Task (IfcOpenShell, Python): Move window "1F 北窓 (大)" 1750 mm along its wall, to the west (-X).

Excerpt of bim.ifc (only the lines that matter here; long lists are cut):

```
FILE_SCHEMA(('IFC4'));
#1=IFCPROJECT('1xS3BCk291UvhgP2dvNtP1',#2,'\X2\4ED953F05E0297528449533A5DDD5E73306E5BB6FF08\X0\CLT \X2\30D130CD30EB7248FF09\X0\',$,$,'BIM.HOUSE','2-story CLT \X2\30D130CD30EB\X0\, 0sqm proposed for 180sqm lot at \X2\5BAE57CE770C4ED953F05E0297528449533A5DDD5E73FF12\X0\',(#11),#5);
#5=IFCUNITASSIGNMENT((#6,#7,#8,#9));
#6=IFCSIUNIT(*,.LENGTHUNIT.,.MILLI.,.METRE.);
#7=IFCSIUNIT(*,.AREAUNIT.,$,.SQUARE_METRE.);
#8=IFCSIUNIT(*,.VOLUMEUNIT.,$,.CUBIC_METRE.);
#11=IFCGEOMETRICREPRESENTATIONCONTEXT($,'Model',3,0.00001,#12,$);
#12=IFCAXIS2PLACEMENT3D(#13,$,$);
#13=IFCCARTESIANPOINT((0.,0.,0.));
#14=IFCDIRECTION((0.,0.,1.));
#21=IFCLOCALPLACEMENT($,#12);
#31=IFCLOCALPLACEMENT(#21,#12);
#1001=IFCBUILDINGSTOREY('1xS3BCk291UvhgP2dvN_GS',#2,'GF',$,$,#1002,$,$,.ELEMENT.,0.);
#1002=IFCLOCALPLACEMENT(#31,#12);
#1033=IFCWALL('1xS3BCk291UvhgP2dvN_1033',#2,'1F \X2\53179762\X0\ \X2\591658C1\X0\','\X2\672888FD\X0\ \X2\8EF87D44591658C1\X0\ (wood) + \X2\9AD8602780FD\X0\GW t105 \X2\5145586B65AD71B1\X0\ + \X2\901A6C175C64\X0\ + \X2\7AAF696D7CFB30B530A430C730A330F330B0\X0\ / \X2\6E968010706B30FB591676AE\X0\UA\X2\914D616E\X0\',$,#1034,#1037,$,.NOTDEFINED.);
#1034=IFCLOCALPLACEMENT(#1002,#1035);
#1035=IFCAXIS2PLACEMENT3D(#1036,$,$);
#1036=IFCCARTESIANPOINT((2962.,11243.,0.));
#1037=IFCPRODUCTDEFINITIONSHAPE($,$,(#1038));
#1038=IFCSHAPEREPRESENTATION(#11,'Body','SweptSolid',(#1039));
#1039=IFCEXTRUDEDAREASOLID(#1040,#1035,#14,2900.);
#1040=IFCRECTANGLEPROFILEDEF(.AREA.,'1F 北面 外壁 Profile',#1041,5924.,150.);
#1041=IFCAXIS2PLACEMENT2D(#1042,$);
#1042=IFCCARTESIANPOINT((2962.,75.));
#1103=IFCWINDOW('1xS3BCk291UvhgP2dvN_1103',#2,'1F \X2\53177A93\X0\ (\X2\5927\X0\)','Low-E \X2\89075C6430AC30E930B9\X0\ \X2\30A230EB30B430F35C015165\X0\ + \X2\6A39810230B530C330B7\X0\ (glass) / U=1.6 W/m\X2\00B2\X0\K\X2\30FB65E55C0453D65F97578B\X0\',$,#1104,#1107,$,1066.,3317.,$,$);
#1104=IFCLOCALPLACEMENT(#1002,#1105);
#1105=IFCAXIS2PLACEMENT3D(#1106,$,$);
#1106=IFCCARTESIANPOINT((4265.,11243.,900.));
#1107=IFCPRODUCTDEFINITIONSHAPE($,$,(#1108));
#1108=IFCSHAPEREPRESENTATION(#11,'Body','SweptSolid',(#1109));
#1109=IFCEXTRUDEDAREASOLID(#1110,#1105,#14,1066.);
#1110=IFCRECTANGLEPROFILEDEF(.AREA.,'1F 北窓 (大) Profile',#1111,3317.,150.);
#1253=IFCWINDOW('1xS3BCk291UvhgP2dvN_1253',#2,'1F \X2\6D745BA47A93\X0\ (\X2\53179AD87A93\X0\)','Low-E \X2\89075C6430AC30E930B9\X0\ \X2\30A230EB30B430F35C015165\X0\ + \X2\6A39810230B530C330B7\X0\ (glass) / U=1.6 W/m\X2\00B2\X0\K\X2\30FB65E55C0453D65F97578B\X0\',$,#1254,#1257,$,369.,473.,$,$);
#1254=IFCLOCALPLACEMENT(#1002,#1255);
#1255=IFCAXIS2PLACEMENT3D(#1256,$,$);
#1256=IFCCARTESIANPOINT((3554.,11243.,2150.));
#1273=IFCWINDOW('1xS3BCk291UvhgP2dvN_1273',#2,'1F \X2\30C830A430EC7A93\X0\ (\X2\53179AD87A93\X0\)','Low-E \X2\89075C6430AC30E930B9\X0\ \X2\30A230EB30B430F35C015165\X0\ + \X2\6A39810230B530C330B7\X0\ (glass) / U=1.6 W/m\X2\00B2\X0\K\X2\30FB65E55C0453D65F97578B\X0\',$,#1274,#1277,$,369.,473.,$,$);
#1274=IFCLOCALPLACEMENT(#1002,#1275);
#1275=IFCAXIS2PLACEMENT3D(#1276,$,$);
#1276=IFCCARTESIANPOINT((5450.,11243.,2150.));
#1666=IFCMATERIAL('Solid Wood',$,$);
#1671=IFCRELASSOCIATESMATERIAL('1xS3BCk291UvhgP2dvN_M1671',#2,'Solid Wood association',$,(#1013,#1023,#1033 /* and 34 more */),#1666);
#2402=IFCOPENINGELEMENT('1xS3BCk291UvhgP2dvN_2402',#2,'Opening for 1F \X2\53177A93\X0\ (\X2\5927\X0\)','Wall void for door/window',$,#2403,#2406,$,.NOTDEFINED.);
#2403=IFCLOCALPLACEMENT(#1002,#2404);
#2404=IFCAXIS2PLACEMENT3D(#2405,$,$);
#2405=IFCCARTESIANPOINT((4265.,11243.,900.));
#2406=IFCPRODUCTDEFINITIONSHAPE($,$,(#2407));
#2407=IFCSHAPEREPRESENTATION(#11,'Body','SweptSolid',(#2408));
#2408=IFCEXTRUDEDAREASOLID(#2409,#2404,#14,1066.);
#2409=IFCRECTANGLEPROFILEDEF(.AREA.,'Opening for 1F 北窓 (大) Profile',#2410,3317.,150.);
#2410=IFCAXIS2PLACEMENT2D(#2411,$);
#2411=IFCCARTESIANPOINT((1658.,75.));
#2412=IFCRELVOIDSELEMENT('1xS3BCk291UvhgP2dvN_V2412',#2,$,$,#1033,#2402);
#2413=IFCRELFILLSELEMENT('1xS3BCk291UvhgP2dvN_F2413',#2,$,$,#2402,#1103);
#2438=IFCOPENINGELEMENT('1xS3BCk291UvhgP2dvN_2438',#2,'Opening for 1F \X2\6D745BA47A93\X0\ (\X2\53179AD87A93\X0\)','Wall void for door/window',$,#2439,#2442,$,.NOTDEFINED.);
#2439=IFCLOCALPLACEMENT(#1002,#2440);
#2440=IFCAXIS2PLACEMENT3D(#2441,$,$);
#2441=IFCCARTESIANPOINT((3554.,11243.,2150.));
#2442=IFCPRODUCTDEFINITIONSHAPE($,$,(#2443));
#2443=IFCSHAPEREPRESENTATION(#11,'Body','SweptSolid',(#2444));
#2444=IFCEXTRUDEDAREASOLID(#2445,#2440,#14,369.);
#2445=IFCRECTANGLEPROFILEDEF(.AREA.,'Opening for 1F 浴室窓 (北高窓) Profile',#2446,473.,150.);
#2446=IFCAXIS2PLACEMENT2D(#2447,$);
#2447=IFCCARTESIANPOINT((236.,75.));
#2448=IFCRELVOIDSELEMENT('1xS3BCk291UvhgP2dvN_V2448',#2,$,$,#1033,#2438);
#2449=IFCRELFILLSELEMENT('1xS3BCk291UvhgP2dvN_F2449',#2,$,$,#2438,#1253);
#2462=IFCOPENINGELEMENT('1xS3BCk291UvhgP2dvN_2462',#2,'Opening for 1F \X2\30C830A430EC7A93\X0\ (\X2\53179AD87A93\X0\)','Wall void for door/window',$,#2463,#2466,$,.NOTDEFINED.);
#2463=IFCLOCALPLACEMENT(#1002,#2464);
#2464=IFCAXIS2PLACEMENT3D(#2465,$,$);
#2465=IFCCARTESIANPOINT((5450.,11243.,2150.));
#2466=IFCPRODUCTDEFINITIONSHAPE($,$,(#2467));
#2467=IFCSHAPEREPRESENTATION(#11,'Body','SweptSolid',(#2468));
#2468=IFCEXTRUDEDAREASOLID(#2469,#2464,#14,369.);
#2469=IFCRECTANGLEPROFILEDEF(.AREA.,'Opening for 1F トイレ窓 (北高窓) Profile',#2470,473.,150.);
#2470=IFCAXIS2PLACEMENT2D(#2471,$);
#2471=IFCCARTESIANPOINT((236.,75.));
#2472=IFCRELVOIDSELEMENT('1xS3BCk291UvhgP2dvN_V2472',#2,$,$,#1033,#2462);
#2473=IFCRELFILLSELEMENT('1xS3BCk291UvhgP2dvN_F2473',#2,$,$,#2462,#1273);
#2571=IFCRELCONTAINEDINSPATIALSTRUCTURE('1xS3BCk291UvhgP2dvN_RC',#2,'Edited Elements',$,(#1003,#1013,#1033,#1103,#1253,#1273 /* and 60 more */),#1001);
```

```python
import ifcopenshell
import ifcopenshell.api.geometry
import ifcopenshell.util.placement
import ifcopenshell.util.unit

model = ifcopenshell.open("bim.ifc")
unit_scale = ifcopenshell.util.unit.calculate_unit_scale(model)

window = model.by_guid("1xS3BCk291UvhgP2dvN_1103")
opening = window.FillsVoids[0].RelatingOpeningElement
wall = opening.VoidsElements[0].RelatingBuildingElement

wall_matrix = ifcopenshell.util.placement.get_local_placement(wall.ObjectPlacement)
shift = wall_matrix[:3, 0] * -1.75 / unit_scale
before = ifcopenshell.util.placement.get_local_placement(window.ObjectPlacement)[:3, 3].copy()

# The window is not placed relative to its opening, so move both.
for product in (opening, window):
    matrix = ifcopenshell.util.placement.get_local_placement(product.ObjectPlacement)
    matrix[:3, 3] += shift
    ifcopenshell.api.geometry.edit_object_placement(model, product=product, matrix=matrix, is_si=False)

after = ifcopenshell.util.placement.get_local_placement(window.ObjectPlacement)[:3, 3]
print("window moved by", (after - before).round(3) + 0.0)

model.write("bim-out.ifc")
```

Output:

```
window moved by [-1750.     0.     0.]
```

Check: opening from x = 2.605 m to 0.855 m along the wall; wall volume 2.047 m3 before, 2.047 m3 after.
